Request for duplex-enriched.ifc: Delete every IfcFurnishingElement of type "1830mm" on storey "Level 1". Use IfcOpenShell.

First a look at what the model holds.

```python
import ifcopenshell
import ifcopenshell.util.element

model = ifcopenshell.open("duplex-enriched.ifc")
print(model.schema)
storey = next(s for s in model.by_type("IfcBuildingStorey") if s.Name == "Level 1")
furniture = [e for e in ifcopenshell.util.element.get_decomposition(storey) if e.is_a("IfcFurnishingElement")]
seen = {}
for e in furniture:
    element_type = ifcopenshell.util.element.get_type(e)
    name = element_type.Name if element_type not in (None, e) else None
    seen[name] = seen.get(name, 0) + 1
for name, count in sorted(seen.items(), key=str):
    print(count, "x", name)
```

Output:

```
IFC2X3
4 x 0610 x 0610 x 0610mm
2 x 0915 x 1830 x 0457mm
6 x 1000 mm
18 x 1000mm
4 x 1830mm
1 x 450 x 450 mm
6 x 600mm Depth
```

```python
import ifcopenshell
import ifcopenshell.api.root
import ifcopenshell.util.element

model = ifcopenshell.open("duplex-enriched.ifc")

storey = next(s for s in model.by_type("IfcBuildingStorey") if s.Name == "Level 1")
furniture = [e for e in ifcopenshell.util.element.get_decomposition(storey) if e.is_a("IfcFurnishingElement")]
targets = [e for e in furniture if (t := ifcopenshell.util.element.get_type(e)) not in (None, e) and t.Name == "1830mm"]

for e in targets:
    ifcopenshell.api.root.remove_product(model, product=e)
print(len(targets), "removed")

model.write("duplex-enriched_updated.ifc")
```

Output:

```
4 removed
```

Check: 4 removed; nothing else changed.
